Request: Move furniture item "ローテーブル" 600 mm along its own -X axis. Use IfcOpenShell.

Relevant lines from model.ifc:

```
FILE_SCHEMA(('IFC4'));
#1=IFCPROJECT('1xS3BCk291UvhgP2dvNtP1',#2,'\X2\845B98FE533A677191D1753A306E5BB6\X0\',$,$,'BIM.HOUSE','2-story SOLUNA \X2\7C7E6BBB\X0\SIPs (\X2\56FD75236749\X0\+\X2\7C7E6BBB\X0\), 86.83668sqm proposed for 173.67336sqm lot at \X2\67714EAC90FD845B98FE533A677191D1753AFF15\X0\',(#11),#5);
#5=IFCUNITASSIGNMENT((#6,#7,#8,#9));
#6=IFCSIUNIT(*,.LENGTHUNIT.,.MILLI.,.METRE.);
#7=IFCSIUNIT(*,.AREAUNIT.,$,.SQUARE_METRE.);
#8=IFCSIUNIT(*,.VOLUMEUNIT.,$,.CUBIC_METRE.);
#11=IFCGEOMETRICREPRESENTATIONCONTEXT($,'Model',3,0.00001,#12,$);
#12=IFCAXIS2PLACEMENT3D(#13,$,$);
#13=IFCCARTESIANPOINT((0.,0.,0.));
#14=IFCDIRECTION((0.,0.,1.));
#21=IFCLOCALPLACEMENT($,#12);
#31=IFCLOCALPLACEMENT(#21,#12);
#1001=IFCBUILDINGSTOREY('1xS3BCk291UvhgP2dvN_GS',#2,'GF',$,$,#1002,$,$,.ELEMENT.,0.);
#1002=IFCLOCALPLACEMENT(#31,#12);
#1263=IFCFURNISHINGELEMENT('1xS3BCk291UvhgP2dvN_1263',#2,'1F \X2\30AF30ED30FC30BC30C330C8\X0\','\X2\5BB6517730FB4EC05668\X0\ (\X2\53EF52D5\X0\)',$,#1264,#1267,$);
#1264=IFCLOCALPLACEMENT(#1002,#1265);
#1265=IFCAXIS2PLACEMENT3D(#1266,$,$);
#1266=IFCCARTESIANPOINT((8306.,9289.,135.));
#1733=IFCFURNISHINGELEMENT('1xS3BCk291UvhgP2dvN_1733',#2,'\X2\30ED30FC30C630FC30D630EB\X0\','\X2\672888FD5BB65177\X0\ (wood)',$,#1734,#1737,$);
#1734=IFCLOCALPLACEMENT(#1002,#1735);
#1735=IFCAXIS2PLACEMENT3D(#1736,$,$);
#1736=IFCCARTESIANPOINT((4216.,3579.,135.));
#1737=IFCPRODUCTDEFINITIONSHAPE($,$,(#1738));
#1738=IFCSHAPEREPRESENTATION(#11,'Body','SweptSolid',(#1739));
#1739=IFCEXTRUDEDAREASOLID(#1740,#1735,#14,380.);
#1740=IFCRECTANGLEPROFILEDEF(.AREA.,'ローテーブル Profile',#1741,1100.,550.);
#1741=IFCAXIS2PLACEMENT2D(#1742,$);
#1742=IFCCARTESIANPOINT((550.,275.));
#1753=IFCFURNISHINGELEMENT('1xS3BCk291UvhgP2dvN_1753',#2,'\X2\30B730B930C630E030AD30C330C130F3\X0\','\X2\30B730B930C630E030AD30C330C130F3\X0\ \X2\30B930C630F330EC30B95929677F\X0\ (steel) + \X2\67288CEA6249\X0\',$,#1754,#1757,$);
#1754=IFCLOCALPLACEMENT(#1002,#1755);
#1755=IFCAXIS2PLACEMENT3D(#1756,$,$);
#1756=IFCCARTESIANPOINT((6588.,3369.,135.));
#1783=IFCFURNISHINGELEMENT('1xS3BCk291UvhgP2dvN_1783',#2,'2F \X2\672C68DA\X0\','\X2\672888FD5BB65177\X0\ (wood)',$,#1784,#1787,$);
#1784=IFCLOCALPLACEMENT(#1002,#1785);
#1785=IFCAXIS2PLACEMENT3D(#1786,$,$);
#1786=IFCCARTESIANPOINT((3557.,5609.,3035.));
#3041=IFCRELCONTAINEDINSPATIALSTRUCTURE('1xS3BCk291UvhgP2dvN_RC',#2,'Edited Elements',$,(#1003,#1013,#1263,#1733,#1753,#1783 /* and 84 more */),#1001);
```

```python
import ifcopenshell
import ifcopenshell.api.geometry
import ifcopenshell.util.placement

model = ifcopenshell.open("model.ifc")

item = model.by_id(1733)
matrix = ifcopenshell.util.placement.get_local_placement(item.ObjectPlacement)
matrix[:3, 3] -= matrix[:3, 0] * 600.0
ifcopenshell.api.geometry.edit_object_placement(model, product=item, matrix=matrix, is_si=False)

print(ifcopenshell.util.placement.get_local_placement(item.ObjectPlacement).round(3) + 0.0)

model.write("model_rev.ifc")
```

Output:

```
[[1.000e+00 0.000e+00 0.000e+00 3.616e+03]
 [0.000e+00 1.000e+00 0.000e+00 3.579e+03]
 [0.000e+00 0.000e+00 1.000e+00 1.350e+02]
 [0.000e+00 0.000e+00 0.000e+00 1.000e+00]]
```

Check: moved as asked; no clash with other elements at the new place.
